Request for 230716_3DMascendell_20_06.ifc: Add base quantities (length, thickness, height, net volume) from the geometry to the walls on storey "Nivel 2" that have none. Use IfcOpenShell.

First a look at what the model holds.

```python
import ifcopenshell
import ifcopenshell.util.element
import ifcopenshell.util.unit

model = ifcopenshell.open("230716_3DMascendell_20_06.ifc")
print(model.schema)
for unit_type in ("LENGTHUNIT", "AREAUNIT", "VOLUMEUNIT"):
    print(unit_type, ifcopenshell.util.unit.calculate_unit_scale(model, unit_type))
storey = next(s for s in model.by_type("IfcBuildingStorey") if s.Name == "Nivel 2")
walls = [e for e in ifcopenshell.util.element.get_decomposition(storey) if e.is_a("IfcWall")]
for e in sorted(walls, key=lambda e: e.id()):
    print(e.id(), e.is_a(), e.Name, list(ifcopenshell.util.element.get_psets(e, qtos_only=True)), sep=" | ")
```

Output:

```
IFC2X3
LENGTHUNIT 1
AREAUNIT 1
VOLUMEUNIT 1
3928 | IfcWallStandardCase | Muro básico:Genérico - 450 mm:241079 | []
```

```python
import ifcopenshell
import ifcopenshell.api.pset
import ifcopenshell.geom
import ifcopenshell.util.element
import ifcopenshell.util.shape
import ifcopenshell.util.unit

model = ifcopenshell.open("230716_3DMascendell_20_06.ifc")
unit_scale = ifcopenshell.util.unit.calculate_unit_scale(model)
volume_scale = ifcopenshell.util.unit.calculate_unit_scale(model, "VOLUMEUNIT")
settings = ifcopenshell.geom.settings()

storey = next(s for s in model.by_type("IfcBuildingStorey") if s.Name == "Nivel 2")
walls = [e for e in ifcopenshell.util.element.get_decomposition(storey) if e.is_a("IfcWall")]

for e in sorted(walls, key=lambda e: e.id()):
    if ifcopenshell.util.element.get_psets(e, qtos_only=True, should_inherit=False):
        continue
    # Geometry comes back in metres, in the element's own axes.
    shape = ifcopenshell.geom.create_shape(settings, e)
    values = {
        "Length": ifcopenshell.util.shape.get_x(shape.geometry) / unit_scale,
        "Width": ifcopenshell.util.shape.get_y(shape.geometry) / unit_scale,
        "Height": ifcopenshell.util.shape.get_z(shape.geometry) / unit_scale,
        "NetVolume": ifcopenshell.util.shape.get_volume(shape.geometry) / volume_scale,
    }
    qto = ifcopenshell.api.pset.add_qto(model, product=e, name="BaseQuantities")
    ifcopenshell.api.pset.edit_qto(model, qto=qto, properties=values)
    print(e.id(), {k: round(v, 3) for k, v in values.items()})

model.write("230716_3DMascendell_20_06_edited.ifc")
```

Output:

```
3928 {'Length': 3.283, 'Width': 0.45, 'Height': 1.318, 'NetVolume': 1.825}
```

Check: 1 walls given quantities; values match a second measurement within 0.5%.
